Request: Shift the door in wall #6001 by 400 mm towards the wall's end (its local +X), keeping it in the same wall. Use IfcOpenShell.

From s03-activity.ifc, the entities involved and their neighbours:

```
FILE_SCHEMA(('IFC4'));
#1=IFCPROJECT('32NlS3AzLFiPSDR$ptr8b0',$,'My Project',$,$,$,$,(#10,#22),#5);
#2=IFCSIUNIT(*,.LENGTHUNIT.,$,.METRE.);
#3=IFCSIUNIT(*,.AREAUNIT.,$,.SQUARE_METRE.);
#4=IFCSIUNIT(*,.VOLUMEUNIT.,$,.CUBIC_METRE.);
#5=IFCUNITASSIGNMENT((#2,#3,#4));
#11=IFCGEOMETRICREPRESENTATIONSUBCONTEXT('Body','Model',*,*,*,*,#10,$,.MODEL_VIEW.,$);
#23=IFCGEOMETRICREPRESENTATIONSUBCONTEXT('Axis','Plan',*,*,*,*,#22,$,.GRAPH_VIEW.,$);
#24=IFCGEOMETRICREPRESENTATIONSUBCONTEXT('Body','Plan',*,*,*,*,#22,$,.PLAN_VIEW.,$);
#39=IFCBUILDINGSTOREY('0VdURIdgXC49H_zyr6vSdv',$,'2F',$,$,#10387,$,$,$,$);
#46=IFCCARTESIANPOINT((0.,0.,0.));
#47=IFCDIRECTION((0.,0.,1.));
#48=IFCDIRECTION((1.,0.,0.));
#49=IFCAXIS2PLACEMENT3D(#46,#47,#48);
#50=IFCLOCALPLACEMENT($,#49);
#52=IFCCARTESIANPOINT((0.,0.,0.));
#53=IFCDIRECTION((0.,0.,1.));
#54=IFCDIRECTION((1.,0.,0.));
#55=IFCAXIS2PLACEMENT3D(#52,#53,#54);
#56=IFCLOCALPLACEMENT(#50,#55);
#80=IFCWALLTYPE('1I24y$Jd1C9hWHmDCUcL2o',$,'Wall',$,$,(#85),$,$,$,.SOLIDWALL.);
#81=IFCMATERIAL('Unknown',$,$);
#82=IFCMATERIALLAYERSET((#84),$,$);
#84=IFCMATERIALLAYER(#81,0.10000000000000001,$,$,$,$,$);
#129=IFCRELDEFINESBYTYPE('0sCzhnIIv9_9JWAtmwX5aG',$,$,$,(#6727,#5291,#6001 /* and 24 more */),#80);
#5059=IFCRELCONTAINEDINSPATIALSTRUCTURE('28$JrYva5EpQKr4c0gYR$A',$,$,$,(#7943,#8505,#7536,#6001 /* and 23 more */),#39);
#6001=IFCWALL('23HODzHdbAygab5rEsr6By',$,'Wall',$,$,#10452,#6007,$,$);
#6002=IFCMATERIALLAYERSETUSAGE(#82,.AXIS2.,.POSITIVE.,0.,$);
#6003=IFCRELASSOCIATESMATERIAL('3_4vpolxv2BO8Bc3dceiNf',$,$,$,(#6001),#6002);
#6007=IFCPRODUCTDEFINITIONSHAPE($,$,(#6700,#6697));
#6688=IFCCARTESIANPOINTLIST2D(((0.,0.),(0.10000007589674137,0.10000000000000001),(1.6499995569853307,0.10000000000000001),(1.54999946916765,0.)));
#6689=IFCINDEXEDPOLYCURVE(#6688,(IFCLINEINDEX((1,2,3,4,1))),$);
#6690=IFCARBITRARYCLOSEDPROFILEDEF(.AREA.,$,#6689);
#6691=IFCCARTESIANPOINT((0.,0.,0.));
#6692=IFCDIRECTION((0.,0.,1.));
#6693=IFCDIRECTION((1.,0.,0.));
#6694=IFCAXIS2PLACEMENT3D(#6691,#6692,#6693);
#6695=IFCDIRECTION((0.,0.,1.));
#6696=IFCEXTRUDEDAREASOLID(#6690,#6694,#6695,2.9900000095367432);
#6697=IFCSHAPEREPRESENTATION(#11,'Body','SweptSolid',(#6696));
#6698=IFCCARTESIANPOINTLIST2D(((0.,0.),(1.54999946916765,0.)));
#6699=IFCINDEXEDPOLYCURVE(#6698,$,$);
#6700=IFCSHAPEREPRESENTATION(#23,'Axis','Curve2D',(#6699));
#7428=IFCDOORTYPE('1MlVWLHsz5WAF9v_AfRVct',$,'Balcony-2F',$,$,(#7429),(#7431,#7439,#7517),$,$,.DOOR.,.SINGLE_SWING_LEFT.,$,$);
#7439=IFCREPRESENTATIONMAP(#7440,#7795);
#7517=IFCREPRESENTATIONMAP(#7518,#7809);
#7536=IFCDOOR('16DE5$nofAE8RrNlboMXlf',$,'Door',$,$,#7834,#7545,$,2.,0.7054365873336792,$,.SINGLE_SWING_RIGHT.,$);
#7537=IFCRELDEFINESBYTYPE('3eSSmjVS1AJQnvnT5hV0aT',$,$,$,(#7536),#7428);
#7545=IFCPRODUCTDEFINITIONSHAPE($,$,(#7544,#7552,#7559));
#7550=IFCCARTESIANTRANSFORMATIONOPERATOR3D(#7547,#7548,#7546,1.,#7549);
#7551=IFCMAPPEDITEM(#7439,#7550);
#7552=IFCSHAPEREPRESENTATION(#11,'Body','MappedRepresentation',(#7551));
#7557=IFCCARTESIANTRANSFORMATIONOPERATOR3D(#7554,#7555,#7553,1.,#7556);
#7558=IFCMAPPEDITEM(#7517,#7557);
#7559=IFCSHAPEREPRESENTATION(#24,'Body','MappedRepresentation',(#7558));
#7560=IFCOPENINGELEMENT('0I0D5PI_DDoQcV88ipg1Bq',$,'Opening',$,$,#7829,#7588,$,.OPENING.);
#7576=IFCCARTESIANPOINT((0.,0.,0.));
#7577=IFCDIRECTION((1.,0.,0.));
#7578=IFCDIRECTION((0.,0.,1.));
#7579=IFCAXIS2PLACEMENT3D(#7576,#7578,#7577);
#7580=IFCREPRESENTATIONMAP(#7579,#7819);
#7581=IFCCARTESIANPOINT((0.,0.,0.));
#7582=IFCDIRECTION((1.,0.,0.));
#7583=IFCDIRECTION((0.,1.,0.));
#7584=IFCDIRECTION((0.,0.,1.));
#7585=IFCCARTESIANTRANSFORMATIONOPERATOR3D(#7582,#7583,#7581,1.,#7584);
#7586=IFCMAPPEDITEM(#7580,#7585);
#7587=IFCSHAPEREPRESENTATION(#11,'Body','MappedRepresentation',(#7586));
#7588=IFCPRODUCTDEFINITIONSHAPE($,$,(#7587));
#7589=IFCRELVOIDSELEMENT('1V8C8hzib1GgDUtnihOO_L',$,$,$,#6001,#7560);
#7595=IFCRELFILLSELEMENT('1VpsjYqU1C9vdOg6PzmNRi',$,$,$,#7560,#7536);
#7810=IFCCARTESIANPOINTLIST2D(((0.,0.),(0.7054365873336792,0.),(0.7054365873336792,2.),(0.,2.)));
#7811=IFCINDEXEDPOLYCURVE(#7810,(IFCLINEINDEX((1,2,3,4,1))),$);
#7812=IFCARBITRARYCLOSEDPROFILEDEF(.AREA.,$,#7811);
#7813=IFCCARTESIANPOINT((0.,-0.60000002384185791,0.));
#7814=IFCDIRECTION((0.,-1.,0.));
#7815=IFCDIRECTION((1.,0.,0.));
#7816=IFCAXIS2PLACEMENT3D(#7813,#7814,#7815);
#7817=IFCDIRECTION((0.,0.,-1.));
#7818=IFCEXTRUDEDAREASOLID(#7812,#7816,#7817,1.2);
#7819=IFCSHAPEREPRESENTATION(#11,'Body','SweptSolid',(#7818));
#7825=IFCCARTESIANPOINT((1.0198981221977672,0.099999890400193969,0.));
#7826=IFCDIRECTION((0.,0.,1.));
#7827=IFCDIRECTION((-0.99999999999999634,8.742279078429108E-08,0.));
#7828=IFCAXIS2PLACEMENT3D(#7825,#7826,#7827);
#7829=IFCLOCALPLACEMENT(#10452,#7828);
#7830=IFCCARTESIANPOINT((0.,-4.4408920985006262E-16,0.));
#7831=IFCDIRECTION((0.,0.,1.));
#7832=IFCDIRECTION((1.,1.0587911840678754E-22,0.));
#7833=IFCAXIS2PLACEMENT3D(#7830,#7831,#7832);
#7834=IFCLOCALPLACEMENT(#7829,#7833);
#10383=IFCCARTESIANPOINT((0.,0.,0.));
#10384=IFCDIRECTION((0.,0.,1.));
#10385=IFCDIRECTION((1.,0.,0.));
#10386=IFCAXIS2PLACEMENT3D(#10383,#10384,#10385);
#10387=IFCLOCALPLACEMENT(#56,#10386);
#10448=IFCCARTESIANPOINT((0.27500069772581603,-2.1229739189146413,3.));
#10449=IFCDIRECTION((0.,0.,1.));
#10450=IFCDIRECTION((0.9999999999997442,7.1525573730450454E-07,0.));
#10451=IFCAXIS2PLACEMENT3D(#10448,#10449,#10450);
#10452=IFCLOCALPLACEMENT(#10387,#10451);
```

```python
import ifcopenshell
import ifcopenshell.api.geometry
import ifcopenshell.util.placement
import ifcopenshell.util.unit

model = ifcopenshell.open("s03-activity.ifc")
unit_scale = ifcopenshell.util.unit.calculate_unit_scale(model)

door = model.by_guid("16DE5$nofAE8RrNlboMXlf")
opening = door.FillsVoids[0].RelatingOpeningElement
wall = opening.VoidsElements[0].RelatingBuildingElement

wall_matrix = ifcopenshell.util.placement.get_local_placement(wall.ObjectPlacement)
shift = wall_matrix[:3, 0] * 0.4 / unit_scale
before = ifcopenshell.util.placement.get_local_placement(door.ObjectPlacement)[:3, 3].copy()

# The door is placed relative to its opening, so it follows when the opening moves.
matrix = ifcopenshell.util.placement.get_local_placement(opening.ObjectPlacement)
matrix[:3, 3] += shift
ifcopenshell.api.geometry.edit_object_placement(
    model, product=opening, matrix=matrix, is_si=False, should_transform_children=True
)

after = ifcopenshell.util.placement.get_local_placement(door.ObjectPlacement)[:3, 3]
print("door moved by", (after - before).round(3) + 0.0)

model.write("s03-activity_v2.ifc")
```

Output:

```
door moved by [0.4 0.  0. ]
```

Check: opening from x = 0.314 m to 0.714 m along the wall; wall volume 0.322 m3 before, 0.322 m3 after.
